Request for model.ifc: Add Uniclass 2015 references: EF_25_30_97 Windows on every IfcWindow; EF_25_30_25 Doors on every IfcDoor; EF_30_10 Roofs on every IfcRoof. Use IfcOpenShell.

First a look at what the model holds.

```python
import ifcopenshell

model = ifcopenshell.open("model.ifc")
print(model.schema)
print("classifications:", [c.Name for c in model.by_type("IfcClassification")])
for ifc_class in ("IfcDoor", "IfcRoof", "IfcStair", "IfcWall", "IfcWindow"):
    print(ifc_class, len(model.by_type(ifc_class)))
```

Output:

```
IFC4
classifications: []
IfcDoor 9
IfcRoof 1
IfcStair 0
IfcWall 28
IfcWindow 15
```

```python
import ifcopenshell
import ifcopenshell.api.classification

model = ifcopenshell.open("model.ifc")

system = ifcopenshell.api.classification.add_classification(model, classification="Uniclass 2015")

codes = {
    "IfcWindow": ("EF_25_30_97", "Windows"),
    "IfcDoor": ("EF_25_30_25", "Doors"),
    "IfcRoof": ("EF_30_10", "Roofs"),
}
for ifc_class, (code, name) in codes.items():
    products = model.by_type(ifc_class)
    ifcopenshell.api.classification.add_reference(
        model, products=products, classification=system, identification=code, name=name
    )
    print(code, len(products))

model.write("model_v2.ifc")
```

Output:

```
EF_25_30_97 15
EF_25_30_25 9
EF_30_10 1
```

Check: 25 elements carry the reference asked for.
